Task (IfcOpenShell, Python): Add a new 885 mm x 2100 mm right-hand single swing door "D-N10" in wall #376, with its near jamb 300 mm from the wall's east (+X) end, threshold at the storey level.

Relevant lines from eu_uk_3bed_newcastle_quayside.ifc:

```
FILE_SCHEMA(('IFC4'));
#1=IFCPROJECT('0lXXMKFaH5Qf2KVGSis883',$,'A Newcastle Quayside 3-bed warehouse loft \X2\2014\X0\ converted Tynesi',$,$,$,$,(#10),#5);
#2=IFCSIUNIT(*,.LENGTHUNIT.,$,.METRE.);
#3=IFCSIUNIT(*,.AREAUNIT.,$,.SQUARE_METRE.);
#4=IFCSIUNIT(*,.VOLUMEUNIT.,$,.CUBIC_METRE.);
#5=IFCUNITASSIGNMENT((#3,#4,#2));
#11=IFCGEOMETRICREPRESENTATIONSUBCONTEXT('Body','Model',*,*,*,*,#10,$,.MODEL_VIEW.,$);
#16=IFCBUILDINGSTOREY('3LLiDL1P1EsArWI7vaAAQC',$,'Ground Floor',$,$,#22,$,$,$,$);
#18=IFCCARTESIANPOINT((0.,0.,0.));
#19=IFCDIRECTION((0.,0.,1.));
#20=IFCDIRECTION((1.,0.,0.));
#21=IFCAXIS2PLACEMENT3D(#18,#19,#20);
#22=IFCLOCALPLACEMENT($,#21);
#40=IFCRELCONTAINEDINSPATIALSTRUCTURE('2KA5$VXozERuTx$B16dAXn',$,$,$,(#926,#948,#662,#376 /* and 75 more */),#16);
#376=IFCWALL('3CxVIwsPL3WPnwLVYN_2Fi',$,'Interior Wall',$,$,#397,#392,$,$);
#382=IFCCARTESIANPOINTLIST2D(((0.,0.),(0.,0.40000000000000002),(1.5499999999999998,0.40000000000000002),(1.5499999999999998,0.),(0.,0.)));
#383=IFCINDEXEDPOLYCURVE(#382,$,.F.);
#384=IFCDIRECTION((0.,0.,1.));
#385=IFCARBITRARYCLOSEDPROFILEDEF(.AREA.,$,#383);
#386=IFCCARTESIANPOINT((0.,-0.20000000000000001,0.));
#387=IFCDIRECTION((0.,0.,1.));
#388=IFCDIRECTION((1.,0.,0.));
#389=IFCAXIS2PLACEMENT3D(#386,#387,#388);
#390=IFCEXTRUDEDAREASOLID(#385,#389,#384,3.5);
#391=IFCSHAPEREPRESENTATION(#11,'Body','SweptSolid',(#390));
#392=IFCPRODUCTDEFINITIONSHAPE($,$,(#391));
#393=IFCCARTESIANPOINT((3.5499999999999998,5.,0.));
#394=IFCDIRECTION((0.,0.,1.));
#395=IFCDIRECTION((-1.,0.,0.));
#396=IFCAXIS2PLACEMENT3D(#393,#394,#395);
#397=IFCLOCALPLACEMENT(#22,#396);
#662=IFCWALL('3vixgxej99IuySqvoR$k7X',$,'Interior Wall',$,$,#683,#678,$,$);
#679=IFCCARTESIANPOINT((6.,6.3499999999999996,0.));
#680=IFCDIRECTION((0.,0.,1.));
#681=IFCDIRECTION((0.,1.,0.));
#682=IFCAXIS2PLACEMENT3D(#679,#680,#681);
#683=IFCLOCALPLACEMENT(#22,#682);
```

```python
import numpy as np
import ifcopenshell
import ifcopenshell.api.feature
import ifcopenshell.api.geometry
import ifcopenshell.api.root
import ifcopenshell.api.spatial
import ifcopenshell.geom
import ifcopenshell.util.element
import ifcopenshell.util.placement
import ifcopenshell.util.representation
import ifcopenshell.util.shape
import ifcopenshell.util.unit

model = ifcopenshell.open("eu_uk_3bed_newcastle_quayside.ifc")
unit_scale = ifcopenshell.util.unit.calculate_unit_scale(model)
settings = ifcopenshell.geom.settings()


def volume(element):
    """Net volume in cubic metres, openings subtracted."""
    shape = ifcopenshell.geom.create_shape(settings, element)
    return ifcopenshell.util.shape.get_volume(shape.geometry)


wall = model.by_guid("3CxVIwsPL3WPnwLVYN_2Fi")
storey = ifcopenshell.util.element.get_container(wall, ifc_class="IfcBuildingStorey")
context = ifcopenshell.util.representation.get_context(model, "Model", "Body", "MODEL_VIEW")
before = volume(wall)

width, height, from_end, sill = 0.885, 2.1, 0.3, 0.0  # metres

# The wall runs along its own X axis, and the end named is its -X end.
wall_shape = ifcopenshell.geom.create_shape(settings, wall)
x, y, z = ifcopenshell.util.shape.get_vertices(wall_shape.geometry).T
start = x.min() + from_end
face, thickness = float(y.min()), float(y.max() - y.min())
wall_matrix = ifcopenshell.util.placement.get_local_placement(wall.ObjectPlacement)
level = ifcopenshell.util.placement.get_local_placement(storey.ObjectPlacement)[2, 3]


def in_wall(x, y):
    """Placement at x, y metres in the wall's axes, at sill height."""
    matrix = wall_matrix.copy()
    matrix[:, 3] = wall_matrix @ np.array([x / unit_scale, y / unit_scale, 0.0, 1.0])
    matrix[2, 3] = level + sill / unit_scale
    return matrix


# Opening: a box that overshoots both wall faces by 50 mm.
opening = ifcopenshell.api.root.create_entity(model, ifc_class="IfcOpeningElement", predefined_type="OPENING")
box = ifcopenshell.api.geometry.add_wall_representation(
    model, context=context, length=width, height=height, thickness=thickness + 0.1
)
ifcopenshell.api.geometry.assign_representation(model, product=opening, representation=box)
ifcopenshell.api.geometry.edit_object_placement(model, product=opening, matrix=in_wall(start, face - 0.05), is_si=False)
ifcopenshell.api.feature.add_feature(model, feature=opening, element=wall)

door = ifcopenshell.api.root.create_entity(model, ifc_class="IfcDoor", name="D-N10", predefined_type="DOOR")
door.OverallWidth, door.OverallHeight = width / unit_scale, height / unit_scale
door.OperationType = "SINGLE_SWING_RIGHT"
body = ifcopenshell.api.geometry.add_door_representation(
    model,
    context=context,
    overall_width=door.OverallWidth,
    overall_height=door.OverallHeight,
    operation_type="SINGLE_SWING_RIGHT",
    lining_properties={"LiningDepth": thickness / unit_scale, "ThresholdDepth": thickness / unit_scale},
)
ifcopenshell.api.geometry.assign_representation(model, product=door, representation=body)
ifcopenshell.api.spatial.assign_container(model, products=[door], relating_structure=storey)
ifcopenshell.api.feature.add_filling(model, opening=opening, element=door)

# The lining spans the wall, so the door starts at the wall face.
ifcopenshell.api.geometry.edit_object_placement(model, product=door, matrix=in_wall(start, face), is_si=False)

after = volume(wall)

print(f"wall volume {before:.3f} -> {after:.3f} m3")

model.write("eu_uk_3bed_newcastle_quayside_v2.ifc")
```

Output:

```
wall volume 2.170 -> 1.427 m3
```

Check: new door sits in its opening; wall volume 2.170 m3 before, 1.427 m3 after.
